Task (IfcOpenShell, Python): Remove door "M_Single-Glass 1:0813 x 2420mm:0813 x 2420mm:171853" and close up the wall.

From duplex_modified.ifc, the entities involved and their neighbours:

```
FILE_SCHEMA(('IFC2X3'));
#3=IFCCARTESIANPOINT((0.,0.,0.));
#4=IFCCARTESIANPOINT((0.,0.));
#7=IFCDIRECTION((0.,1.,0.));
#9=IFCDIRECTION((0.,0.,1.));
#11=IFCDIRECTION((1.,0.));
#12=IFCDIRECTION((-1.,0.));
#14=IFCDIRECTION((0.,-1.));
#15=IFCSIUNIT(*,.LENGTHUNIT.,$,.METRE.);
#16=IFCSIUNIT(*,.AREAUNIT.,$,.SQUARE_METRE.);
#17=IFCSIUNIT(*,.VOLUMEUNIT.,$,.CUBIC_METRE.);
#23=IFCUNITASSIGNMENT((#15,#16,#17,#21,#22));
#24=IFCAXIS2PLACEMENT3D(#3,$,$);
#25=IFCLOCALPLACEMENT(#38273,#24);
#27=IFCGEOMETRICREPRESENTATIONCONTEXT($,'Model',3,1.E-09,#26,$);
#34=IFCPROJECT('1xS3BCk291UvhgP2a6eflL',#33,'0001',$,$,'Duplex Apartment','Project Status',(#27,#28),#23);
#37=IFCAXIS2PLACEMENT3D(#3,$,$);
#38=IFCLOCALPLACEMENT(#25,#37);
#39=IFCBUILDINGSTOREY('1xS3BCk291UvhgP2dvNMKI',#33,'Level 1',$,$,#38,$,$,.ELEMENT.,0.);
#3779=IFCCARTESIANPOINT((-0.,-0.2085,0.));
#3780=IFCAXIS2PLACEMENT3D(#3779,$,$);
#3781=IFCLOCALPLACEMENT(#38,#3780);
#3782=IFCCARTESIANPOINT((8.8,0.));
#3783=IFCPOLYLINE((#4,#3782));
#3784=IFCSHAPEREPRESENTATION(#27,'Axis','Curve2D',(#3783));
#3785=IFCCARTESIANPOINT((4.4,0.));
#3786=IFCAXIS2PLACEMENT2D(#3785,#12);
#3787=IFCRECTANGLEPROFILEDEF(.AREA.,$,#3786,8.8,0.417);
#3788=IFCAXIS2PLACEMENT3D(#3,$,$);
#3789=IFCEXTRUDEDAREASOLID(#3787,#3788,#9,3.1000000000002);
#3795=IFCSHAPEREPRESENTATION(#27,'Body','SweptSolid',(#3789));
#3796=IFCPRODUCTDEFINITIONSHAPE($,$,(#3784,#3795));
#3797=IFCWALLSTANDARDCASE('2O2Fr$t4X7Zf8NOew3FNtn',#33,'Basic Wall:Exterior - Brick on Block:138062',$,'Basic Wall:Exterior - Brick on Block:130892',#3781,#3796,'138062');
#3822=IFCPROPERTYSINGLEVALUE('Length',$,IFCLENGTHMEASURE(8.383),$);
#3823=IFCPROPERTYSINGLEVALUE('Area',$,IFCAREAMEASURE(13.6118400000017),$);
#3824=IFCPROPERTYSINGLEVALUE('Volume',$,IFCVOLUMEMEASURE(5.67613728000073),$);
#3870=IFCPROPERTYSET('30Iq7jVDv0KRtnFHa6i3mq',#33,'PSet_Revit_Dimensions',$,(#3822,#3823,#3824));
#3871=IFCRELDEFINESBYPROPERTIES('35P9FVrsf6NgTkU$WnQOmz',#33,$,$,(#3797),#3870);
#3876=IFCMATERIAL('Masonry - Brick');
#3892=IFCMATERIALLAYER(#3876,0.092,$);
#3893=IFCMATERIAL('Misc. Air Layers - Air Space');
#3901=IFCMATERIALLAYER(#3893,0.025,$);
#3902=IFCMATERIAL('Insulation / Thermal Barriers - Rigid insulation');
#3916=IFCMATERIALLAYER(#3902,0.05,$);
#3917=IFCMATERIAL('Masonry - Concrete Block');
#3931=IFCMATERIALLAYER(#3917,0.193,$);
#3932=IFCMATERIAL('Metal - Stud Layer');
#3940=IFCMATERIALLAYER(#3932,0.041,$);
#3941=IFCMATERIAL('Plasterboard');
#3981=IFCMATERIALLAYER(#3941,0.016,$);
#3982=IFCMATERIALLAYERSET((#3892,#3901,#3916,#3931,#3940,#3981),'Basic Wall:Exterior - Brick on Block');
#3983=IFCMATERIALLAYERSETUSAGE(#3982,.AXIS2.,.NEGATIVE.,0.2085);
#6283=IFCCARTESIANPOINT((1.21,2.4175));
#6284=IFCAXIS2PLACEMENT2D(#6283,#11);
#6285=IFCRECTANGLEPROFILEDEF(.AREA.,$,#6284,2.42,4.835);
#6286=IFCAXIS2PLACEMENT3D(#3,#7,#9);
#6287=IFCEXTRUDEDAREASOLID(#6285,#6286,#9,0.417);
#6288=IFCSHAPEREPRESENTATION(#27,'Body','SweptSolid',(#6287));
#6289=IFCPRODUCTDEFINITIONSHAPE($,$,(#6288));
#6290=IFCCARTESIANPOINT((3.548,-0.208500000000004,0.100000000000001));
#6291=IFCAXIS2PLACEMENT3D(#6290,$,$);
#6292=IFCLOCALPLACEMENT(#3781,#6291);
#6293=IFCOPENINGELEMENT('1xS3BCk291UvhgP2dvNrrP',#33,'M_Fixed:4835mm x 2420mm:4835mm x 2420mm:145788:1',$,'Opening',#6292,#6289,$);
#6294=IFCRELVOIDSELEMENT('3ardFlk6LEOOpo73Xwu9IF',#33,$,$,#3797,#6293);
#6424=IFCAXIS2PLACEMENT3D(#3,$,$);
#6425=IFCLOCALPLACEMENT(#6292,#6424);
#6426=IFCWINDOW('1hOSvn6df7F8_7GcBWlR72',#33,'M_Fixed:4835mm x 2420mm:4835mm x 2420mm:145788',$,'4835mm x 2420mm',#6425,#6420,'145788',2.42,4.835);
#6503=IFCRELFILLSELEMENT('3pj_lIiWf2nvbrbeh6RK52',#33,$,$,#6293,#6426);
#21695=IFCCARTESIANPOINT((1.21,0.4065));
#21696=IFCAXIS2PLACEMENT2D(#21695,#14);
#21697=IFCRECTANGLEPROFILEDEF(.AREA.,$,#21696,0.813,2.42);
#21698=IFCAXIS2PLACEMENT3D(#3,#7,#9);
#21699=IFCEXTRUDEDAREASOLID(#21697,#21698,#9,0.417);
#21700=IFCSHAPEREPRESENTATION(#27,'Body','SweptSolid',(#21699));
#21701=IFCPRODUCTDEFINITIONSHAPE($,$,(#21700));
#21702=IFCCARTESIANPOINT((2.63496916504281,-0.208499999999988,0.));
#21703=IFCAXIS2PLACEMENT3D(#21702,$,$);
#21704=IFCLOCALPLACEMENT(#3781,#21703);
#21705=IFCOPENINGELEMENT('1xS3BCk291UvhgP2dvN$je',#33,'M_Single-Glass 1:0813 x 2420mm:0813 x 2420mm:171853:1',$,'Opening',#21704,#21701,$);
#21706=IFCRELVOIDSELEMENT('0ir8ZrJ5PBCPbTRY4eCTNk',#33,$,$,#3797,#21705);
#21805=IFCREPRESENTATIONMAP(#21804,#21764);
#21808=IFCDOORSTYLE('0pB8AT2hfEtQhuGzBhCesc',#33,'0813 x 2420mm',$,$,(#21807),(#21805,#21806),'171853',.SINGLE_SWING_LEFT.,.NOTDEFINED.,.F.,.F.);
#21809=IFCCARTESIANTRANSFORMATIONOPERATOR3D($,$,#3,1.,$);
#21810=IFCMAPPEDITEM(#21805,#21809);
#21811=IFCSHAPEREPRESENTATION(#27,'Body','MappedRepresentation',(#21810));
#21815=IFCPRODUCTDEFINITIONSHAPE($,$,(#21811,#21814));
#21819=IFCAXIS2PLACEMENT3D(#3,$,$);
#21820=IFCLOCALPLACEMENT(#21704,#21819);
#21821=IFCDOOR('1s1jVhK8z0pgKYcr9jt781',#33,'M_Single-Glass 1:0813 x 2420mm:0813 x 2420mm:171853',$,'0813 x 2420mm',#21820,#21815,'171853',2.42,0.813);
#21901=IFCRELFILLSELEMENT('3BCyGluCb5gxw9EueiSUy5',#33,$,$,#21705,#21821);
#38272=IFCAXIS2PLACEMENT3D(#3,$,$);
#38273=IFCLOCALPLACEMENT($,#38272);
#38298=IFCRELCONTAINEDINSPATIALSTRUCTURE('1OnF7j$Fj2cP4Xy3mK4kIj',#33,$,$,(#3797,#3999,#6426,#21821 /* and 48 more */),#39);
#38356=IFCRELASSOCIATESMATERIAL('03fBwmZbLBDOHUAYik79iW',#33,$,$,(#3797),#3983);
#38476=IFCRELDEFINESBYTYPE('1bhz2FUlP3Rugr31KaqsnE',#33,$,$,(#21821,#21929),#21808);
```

```python
import ifcopenshell
import ifcopenshell.api.feature
import ifcopenshell.api.pset
import ifcopenshell.api.root
import ifcopenshell.geom
import ifcopenshell.util.element
import ifcopenshell.util.shape
import ifcopenshell.util.unit

model = ifcopenshell.open("duplex_modified.ifc")
area_scale = ifcopenshell.util.unit.calculate_unit_scale(model, "AREAUNIT")
volume_scale = ifcopenshell.util.unit.calculate_unit_scale(model, "VOLUMEUNIT")
settings = ifcopenshell.geom.settings()


def volume(element):
    """Net volume in cubic metres, openings subtracted."""
    shape = ifcopenshell.geom.create_shape(settings, element)
    return ifcopenshell.util.shape.get_volume(shape.geometry)


door = model.by_id(21821)
opening = door.FillsVoids[0].RelatingOpeningElement
wall = opening.VoidsElements[0].RelatingBuildingElement
before = volume(wall)

ifcopenshell.api.root.remove_product(model, product=door)
ifcopenshell.api.feature.remove_feature(model, feature=opening)

after = volume(wall)
thickness = 0.417  # wall thickness in metres

# Update the wall's stored quantities.
pset = model.by_id(ifcopenshell.util.element.get_pset(wall, "PSet_Revit_Dimensions", should_inherit=False)["id"])
ifcopenshell.api.pset.edit_pset(model, pset=pset, properties={
    "Area": model.create_entity("IfcAreaMeasure", after / thickness / area_scale),
    "Volume": model.create_entity("IfcVolumeMeasure", after / volume_scale),
})

print(f"wall volume {before:.3f} -> {after:.3f} m3")

model.write("duplex_modified_edited.ifc")
```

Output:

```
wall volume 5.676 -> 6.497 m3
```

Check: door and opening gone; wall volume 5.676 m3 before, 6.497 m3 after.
